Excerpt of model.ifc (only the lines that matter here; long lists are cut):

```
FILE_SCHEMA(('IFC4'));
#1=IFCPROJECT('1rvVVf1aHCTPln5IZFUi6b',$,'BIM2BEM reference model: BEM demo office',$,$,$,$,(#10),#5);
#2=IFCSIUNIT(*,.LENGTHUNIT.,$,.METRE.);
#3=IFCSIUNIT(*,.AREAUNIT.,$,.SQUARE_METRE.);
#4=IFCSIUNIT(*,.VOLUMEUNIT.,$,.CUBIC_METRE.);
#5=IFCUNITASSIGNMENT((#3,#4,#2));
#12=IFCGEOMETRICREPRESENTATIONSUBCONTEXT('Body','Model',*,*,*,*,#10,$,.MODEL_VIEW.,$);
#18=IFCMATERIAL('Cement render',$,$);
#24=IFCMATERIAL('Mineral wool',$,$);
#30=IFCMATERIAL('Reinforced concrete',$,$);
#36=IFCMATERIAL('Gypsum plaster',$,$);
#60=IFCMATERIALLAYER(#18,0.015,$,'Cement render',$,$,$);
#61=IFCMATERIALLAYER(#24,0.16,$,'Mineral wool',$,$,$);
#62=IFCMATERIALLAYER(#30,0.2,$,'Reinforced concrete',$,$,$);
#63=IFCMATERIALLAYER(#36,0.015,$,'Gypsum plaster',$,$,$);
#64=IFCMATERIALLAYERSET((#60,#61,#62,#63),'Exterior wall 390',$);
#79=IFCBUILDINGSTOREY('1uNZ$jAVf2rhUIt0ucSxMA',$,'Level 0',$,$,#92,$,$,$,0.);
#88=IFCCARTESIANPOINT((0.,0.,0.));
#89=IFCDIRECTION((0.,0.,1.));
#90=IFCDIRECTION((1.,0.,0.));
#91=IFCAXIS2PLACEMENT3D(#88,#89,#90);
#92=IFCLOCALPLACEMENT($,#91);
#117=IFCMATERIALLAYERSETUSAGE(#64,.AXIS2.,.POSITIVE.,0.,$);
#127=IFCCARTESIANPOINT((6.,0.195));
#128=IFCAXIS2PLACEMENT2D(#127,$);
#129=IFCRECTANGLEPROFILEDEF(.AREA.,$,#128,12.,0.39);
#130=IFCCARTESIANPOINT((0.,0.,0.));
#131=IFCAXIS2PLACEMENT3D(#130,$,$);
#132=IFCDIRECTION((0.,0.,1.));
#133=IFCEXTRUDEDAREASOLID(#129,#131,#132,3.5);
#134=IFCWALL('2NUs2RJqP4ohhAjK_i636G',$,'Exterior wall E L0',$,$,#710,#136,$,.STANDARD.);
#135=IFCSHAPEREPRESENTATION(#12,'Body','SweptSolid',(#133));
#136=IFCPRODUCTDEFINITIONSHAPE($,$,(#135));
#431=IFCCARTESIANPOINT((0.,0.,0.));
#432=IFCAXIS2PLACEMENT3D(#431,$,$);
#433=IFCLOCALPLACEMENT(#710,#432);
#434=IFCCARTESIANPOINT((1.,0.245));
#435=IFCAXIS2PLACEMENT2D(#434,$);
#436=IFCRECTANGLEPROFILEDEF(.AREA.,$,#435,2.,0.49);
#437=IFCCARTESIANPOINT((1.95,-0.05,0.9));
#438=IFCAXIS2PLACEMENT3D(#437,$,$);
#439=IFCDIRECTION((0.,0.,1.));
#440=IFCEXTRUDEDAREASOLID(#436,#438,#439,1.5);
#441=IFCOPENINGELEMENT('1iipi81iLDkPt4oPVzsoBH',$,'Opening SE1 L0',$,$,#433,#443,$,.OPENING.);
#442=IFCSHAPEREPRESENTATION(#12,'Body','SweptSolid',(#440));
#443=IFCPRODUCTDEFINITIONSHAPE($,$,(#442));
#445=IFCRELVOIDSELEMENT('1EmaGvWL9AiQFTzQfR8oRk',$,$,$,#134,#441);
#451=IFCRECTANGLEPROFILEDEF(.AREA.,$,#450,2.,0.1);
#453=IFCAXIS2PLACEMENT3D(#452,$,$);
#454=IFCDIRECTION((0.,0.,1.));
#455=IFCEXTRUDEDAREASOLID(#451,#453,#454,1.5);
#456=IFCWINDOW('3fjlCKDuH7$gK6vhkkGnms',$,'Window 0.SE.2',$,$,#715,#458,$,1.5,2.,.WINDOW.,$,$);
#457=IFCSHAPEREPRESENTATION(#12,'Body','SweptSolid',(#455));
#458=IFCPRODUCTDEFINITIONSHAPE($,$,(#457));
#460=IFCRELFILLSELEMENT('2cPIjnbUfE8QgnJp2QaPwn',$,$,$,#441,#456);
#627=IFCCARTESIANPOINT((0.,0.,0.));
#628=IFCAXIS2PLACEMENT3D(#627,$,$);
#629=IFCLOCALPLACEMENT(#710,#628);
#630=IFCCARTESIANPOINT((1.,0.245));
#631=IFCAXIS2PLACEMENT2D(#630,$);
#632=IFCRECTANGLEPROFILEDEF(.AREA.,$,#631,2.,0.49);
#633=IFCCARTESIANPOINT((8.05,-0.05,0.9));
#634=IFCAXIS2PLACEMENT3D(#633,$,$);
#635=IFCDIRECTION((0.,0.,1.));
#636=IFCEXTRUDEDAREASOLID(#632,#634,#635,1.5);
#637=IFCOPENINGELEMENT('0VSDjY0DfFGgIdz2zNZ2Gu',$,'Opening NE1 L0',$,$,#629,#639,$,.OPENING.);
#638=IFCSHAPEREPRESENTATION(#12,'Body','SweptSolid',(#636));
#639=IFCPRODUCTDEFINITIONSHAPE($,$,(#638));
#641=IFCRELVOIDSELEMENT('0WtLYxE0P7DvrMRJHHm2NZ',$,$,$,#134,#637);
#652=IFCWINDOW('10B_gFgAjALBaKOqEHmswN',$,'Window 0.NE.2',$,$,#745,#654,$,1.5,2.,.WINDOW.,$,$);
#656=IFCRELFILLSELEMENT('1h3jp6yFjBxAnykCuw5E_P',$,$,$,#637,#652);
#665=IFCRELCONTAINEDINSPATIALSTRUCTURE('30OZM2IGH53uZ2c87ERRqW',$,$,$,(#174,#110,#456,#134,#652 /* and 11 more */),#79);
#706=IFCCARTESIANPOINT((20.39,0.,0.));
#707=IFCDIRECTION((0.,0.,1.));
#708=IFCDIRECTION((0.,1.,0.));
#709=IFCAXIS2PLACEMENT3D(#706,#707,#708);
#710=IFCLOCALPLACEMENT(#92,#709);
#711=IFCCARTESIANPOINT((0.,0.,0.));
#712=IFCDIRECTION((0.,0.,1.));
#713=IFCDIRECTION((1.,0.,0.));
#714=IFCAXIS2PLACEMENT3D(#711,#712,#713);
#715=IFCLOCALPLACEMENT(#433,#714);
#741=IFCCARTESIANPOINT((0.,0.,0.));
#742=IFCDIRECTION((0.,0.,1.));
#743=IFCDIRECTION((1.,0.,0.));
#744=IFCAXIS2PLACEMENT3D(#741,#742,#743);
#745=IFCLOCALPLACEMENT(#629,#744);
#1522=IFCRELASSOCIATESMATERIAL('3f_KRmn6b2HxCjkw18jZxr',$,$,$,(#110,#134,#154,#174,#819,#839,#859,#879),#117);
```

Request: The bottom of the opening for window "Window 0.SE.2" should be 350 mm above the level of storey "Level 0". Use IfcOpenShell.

```python
import numpy as np
import ifcopenshell
import ifcopenshell.api.geometry
import ifcopenshell.geom
import ifcopenshell.util.element
import ifcopenshell.util.placement
import ifcopenshell.util.shape
import ifcopenshell.util.unit

model = ifcopenshell.open("model.ifc")
unit_scale = ifcopenshell.util.unit.calculate_unit_scale(model)

window = model.by_guid("3fjlCKDuH7$gK6vhkkGnms")
opening = window.FillsVoids[0].RelatingOpeningElement
storey = ifcopenshell.util.element.get_container(window, ifc_class="IfcBuildingStorey")
level = ifcopenshell.util.placement.get_local_placement(storey.ObjectPlacement)[2, 3]

# The opening's origin need not be at the sill, so measure its lowest point.
shape = ifcopenshell.geom.create_shape(ifcopenshell.geom.settings(), opening)
bottom = ifcopenshell.util.shape.get_shape_bottom_elevation(shape, shape.geometry) / unit_scale
dz = level + 0.35 - bottom

shift = np.array([0.0, 0.0, dz])
# The window is placed relative to its opening, so it follows when the opening moves.
matrix = ifcopenshell.util.placement.get_local_placement(opening.ObjectPlacement)
matrix[:3, 3] += shift
ifcopenshell.api.geometry.edit_object_placement(
    model, product=opening, matrix=matrix, is_si=False, should_transform_children=True
)

print(f"moved by {dz * unit_scale:+.3f} m")

model.write("model_edited.ifc")
```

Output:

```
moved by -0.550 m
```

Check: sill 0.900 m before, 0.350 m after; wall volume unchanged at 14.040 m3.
